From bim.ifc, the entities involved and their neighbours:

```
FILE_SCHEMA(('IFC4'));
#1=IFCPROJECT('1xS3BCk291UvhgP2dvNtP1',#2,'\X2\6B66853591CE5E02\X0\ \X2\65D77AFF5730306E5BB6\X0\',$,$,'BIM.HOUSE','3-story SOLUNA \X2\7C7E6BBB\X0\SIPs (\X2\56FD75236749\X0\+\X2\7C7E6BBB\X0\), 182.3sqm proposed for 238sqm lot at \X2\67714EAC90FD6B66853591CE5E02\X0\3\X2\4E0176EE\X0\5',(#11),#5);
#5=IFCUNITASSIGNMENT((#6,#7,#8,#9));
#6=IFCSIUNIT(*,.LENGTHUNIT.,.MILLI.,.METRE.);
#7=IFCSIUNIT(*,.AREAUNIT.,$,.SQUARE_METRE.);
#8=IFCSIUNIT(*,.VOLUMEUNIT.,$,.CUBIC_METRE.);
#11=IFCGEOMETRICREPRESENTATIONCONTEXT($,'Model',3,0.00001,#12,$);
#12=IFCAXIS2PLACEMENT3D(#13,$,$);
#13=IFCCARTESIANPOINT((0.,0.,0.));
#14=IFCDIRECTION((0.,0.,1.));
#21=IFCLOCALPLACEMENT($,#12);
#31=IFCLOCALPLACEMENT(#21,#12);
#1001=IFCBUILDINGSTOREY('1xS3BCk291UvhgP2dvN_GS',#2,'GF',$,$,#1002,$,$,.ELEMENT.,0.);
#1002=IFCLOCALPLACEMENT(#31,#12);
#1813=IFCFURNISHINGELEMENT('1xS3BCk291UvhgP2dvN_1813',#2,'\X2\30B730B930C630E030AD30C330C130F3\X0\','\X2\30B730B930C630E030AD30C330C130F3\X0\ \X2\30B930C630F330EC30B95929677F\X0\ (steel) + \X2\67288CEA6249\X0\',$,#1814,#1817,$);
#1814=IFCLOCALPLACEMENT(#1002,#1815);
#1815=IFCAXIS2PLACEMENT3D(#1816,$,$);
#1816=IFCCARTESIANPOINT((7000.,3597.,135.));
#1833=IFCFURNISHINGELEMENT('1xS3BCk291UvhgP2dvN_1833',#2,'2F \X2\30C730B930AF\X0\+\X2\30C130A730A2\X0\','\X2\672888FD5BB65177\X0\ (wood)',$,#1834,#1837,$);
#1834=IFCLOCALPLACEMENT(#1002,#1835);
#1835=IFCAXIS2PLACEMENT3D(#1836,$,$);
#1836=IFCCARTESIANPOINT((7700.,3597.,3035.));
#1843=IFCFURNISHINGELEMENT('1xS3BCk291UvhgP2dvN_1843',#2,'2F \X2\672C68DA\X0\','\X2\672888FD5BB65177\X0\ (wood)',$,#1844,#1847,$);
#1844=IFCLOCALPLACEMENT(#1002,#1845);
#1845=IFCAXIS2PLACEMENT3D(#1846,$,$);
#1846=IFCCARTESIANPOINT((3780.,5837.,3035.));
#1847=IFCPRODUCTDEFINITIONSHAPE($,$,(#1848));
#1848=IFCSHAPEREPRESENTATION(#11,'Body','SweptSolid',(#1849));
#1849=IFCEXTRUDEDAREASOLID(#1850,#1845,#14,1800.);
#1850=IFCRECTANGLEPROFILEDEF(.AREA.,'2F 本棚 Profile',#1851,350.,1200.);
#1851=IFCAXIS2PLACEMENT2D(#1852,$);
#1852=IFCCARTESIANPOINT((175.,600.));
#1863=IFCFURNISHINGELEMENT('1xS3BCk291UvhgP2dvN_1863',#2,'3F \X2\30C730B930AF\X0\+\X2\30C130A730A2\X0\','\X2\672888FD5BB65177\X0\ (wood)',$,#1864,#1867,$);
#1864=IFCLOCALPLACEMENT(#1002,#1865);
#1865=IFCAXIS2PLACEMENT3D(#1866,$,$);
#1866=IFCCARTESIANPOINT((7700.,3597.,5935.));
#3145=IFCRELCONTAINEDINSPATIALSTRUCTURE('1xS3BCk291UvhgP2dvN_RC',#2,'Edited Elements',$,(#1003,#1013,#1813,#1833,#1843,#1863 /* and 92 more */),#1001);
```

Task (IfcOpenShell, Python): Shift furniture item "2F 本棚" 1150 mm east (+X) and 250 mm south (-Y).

```python
import ifcopenshell
import ifcopenshell.api.geometry
import ifcopenshell.util.placement
import ifcopenshell.util.unit

model = ifcopenshell.open("bim.ifc")
unit_scale = ifcopenshell.util.unit.calculate_unit_scale(model)

item = model.by_guid("1xS3BCk291UvhgP2dvN_1843")
matrix = ifcopenshell.util.placement.get_local_placement(item.ObjectPlacement)
matrix[0, 3] += 1.15 / unit_scale
matrix[1, 3] -= 0.25 / unit_scale
ifcopenshell.api.geometry.edit_object_placement(model, product=item, matrix=matrix, is_si=False)

print(ifcopenshell.util.placement.get_local_placement(item.ObjectPlacement).round(3) + 0.0)

model.write("bim_updated.ifc")
```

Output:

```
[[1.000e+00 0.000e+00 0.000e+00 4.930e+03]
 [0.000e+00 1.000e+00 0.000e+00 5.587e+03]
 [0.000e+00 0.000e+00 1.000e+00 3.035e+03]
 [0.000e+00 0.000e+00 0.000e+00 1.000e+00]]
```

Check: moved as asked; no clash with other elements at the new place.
